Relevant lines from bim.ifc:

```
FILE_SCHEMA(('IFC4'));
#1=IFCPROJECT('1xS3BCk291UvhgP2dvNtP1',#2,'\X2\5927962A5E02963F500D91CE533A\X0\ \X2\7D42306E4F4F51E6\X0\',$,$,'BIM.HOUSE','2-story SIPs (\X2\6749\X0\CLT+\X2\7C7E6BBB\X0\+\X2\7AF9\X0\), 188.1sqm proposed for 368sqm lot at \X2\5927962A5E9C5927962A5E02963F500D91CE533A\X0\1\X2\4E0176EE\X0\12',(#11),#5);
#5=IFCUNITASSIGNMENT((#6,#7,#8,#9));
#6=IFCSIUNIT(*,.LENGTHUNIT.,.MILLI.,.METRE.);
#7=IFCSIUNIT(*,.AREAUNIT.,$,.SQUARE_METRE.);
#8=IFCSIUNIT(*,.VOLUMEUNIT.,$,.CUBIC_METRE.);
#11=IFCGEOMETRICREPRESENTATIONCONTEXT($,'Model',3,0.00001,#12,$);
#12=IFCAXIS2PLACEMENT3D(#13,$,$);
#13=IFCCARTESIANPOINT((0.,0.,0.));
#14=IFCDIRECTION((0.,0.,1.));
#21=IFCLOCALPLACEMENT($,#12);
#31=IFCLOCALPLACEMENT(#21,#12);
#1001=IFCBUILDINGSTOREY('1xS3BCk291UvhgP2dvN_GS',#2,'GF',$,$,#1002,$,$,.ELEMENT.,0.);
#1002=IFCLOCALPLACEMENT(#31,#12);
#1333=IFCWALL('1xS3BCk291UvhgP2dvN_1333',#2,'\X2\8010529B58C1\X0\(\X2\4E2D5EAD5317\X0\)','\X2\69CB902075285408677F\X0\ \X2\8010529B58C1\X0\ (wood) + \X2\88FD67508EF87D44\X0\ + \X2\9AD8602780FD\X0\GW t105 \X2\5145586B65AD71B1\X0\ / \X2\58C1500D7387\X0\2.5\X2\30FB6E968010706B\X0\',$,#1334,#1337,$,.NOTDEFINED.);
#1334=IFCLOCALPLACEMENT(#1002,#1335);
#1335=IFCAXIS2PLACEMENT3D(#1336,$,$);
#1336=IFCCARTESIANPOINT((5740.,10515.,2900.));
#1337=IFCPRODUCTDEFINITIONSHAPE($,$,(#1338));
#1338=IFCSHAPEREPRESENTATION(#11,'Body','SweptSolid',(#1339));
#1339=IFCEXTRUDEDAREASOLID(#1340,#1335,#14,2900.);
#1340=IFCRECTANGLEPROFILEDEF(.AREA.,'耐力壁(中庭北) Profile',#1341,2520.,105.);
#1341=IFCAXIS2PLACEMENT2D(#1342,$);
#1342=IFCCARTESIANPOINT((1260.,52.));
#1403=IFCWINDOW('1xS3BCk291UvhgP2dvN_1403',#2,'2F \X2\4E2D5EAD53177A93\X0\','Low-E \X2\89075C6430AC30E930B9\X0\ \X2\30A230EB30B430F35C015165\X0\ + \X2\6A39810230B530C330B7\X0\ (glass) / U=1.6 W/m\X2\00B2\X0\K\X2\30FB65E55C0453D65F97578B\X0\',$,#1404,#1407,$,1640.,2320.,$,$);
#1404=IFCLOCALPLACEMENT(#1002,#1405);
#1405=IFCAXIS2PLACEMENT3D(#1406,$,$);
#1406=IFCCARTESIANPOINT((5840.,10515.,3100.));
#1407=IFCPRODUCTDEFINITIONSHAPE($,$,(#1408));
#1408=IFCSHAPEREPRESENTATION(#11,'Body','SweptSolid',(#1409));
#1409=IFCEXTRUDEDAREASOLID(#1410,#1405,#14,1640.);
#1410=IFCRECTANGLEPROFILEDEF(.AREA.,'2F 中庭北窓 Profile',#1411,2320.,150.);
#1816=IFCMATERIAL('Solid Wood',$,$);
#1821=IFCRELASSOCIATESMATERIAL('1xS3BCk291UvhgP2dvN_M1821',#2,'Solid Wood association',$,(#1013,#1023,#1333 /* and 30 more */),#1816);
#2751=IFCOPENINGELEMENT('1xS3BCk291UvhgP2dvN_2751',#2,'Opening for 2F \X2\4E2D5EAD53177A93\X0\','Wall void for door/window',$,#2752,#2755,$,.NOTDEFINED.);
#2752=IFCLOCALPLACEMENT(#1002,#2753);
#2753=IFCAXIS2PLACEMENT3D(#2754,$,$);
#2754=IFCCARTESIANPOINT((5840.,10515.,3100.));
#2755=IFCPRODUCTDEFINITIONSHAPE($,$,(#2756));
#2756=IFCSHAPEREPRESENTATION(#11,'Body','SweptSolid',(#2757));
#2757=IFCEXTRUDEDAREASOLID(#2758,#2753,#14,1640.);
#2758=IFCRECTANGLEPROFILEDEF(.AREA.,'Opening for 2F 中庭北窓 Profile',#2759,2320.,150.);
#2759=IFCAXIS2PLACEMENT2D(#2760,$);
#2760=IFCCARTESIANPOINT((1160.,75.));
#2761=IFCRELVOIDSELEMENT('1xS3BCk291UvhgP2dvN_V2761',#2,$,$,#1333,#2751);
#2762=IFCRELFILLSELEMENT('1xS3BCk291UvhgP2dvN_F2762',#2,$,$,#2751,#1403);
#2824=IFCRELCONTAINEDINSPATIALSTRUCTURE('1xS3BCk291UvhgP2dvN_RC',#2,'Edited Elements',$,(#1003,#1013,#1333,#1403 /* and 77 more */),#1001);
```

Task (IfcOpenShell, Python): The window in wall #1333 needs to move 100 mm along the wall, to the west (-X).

```python
import ifcopenshell
import ifcopenshell.api.geometry
import ifcopenshell.util.placement

model = ifcopenshell.open("bim.ifc")

window = model.by_id(1403)
opening = window.FillsVoids[0].RelatingOpeningElement
wall = opening.VoidsElements[0].RelatingBuildingElement

wall_matrix = ifcopenshell.util.placement.get_local_placement(wall.ObjectPlacement)
shift = wall_matrix[:3, 0] * -100.0
before = ifcopenshell.util.placement.get_local_placement(window.ObjectPlacement)[:3, 3].copy()

# The window is not placed relative to its opening, so move both.
for product in (opening, window):
    matrix = ifcopenshell.util.placement.get_local_placement(product.ObjectPlacement)
    matrix[:3, 3] += shift
    ifcopenshell.api.geometry.edit_object_placement(model, product=product, matrix=matrix, is_si=False)

after = ifcopenshell.util.placement.get_local_placement(window.ObjectPlacement)[:3, 3]
print("window moved by", (after - before).round(3) + 0.0)

model.write("bim_updated.ifc")
```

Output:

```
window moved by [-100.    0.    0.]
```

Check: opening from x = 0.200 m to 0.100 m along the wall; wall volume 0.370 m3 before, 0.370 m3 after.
